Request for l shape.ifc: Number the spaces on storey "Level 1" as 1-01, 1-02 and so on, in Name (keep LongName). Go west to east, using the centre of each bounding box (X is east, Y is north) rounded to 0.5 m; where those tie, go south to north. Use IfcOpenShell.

First a look at what the model holds.

```python
import ifcopenshell
import ifcopenshell.util.element
import ifcopenshell.util.placement

model = ifcopenshell.open("l shape.ifc")
print(model.schema)
storey = next(s for s in model.by_type("IfcBuildingStorey") if s.Name == "Level 1")
spaces = [e for e in ifcopenshell.util.element.get_decomposition(storey) if e.is_a("IfcSpace")]
for e in sorted(spaces, key=lambda e: e.id()):
    origin = ifcopenshell.util.placement.get_local_placement(e.ObjectPlacement)[:3, 3]
    print(e.id(), e.Name, e.LongName, origin.round(2) + 0.0, sep=" | ")
```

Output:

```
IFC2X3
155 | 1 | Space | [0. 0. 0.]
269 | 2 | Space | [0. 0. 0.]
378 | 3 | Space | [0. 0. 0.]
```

```python
import ifcopenshell
import ifcopenshell.geom
import ifcopenshell.util.element
import ifcopenshell.util.shape

model = ifcopenshell.open("l shape.ifc")
settings = ifcopenshell.geom.settings()
settings.set("use-world-coords", True)


def centre(element):
    shape = ifcopenshell.geom.create_shape(settings, element)
    return ifcopenshell.util.shape.get_bbox_centroid(shape.geometry)


storey = next(s for s in model.by_type("IfcBuildingStorey") if s.Name == "Level 1")
spaces = [e for e in ifcopenshell.util.element.get_decomposition(storey) if e.is_a("IfcSpace")]

# Insertion points can sit at a corner or the storey origin, so sort by the geometry (in metres).
centres = {e: centre(e) for e in spaces}
spaces.sort(key=lambda e: (round(centres[e][0] / 0.5), centres[e][1]))

for i, e in enumerate(spaces, start=1):
    number = f"1-{i:02d}"
    e.Name = number
    print(e.id(), number)

model.write("l shape_edited.ifc")
```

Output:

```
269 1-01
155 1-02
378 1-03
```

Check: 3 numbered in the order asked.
